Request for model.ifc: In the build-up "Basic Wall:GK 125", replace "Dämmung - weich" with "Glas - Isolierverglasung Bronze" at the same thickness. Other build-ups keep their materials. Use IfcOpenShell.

First a look at what the model holds.

```python
import ifcopenshell
import ifcopenshell.util.element

model = ifcopenshell.open("model.ifc")
print(model.schema)
for layer_set in model.by_type("IfcMaterialLayerSet"):
    if layer_set.LayerSetName == "Basic Wall:GK 125":
        for layer in layer_set.MaterialLayers:
            print(layer.id(), layer.Material and layer.Material.Name, layer.LayerThickness, sep=" | ")
        print(len(ifcopenshell.util.element.get_elements_by_material(model, layer_set)), "elements and types use it")
print(sorted(m.Name for m in model.by_type("IfcMaterial") if m.Name)[:60])
```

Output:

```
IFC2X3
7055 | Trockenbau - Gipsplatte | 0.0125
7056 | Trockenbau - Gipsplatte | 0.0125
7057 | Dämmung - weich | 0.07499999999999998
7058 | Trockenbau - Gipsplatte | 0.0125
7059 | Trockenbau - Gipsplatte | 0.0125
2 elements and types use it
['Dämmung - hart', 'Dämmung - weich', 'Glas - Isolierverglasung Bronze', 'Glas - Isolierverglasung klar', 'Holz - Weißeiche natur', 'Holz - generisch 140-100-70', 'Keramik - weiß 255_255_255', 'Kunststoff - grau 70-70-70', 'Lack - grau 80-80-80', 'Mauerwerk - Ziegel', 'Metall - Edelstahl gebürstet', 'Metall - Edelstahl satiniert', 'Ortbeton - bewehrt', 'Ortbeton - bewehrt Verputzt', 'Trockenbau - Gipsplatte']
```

```python
import ifcopenshell
import ifcopenshell.api.material

model = ifcopenshell.open("model.ifc")

layer_set = next(s for s in model.by_type("IfcMaterialLayerSet") if s.LayerSetName == "Basic Wall:GK 125")
layer = next(l for l in layer_set.MaterialLayers if l.Material and l.Material.Name == "Dämmung - weich")
material = next(m for m in model.by_type("IfcMaterial") if m.Name == "Glas - Isolierverglasung Bronze")

# Point this one layer at the other material; renaming the old one would change it everywhere.
ifcopenshell.api.material.edit_layer(model, layer=layer, attributes={}, material=material)

print([l.Material.Name if l.Material else None for l in layer_set.MaterialLayers])

model.write("model-out.ifc")
```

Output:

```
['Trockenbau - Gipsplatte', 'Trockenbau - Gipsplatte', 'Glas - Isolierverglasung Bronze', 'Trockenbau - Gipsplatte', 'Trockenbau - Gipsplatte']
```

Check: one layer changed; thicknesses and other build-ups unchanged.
